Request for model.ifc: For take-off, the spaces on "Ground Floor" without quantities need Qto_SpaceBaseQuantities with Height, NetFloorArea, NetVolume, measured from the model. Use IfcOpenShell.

First a look at what the model holds.

```python
import ifcopenshell
import ifcopenshell.util.element
import ifcopenshell.util.unit

model = ifcopenshell.open("model.ifc")
print(model.schema)
for unit_type in ("LENGTHUNIT", "AREAUNIT", "VOLUMEUNIT"):
    print(unit_type, ifcopenshell.util.unit.calculate_unit_scale(model, unit_type))
storey = next(s for s in model.by_type("IfcBuildingStorey") if s.Name == "Ground Floor")
spaces = [e for e in ifcopenshell.util.element.get_decomposition(storey) if e.is_a("IfcSpace")]
for e in sorted(spaces, key=lambda e: e.id()):
    print(e.id(), e.is_a(), e.Name, list(ifcopenshell.util.element.get_psets(e, qtos_only=True)), sep=" | ")
```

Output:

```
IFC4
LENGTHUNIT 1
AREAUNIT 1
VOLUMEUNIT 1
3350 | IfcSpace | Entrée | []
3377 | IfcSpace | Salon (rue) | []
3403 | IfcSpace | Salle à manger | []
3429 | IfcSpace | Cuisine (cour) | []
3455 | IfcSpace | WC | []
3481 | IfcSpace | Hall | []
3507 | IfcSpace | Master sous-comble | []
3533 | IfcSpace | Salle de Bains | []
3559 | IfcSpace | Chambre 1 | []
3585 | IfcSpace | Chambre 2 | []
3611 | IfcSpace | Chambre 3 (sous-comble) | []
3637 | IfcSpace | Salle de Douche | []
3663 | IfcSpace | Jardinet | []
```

```python
import ifcopenshell
import ifcopenshell.api.pset
import ifcopenshell.geom
import ifcopenshell.util.element
import ifcopenshell.util.shape
import ifcopenshell.util.unit

model = ifcopenshell.open("model.ifc")
unit_scale = ifcopenshell.util.unit.calculate_unit_scale(model)
area_scale = ifcopenshell.util.unit.calculate_unit_scale(model, "AREAUNIT")
volume_scale = ifcopenshell.util.unit.calculate_unit_scale(model, "VOLUMEUNIT")
settings = ifcopenshell.geom.settings()

storey = next(s for s in model.by_type("IfcBuildingStorey") if s.Name == "Ground Floor")
spaces = [e for e in ifcopenshell.util.element.get_decomposition(storey) if e.is_a("IfcSpace")]

for e in sorted(spaces, key=lambda e: e.id()):
    if ifcopenshell.util.element.get_psets(e, qtos_only=True, should_inherit=False):
        continue
    # Geometry comes back in metres, in the element's own axes.
    shape = ifcopenshell.geom.create_shape(settings, e)
    values = {
        "Height": ifcopenshell.util.shape.get_z(shape.geometry) / unit_scale,
        "NetFloorArea": ifcopenshell.util.shape.get_footprint_area(shape.geometry) / area_scale,
        "NetVolume": ifcopenshell.util.shape.get_volume(shape.geometry) / volume_scale,
    }
    qto = ifcopenshell.api.pset.add_qto(model, product=e, name="Qto_SpaceBaseQuantities")
    ifcopenshell.api.pset.edit_qto(model, qto=qto, properties=values)
    print(e.id(), {k: round(v, 3) for k, v in values.items()})

model.write("model_updated.ifc")
```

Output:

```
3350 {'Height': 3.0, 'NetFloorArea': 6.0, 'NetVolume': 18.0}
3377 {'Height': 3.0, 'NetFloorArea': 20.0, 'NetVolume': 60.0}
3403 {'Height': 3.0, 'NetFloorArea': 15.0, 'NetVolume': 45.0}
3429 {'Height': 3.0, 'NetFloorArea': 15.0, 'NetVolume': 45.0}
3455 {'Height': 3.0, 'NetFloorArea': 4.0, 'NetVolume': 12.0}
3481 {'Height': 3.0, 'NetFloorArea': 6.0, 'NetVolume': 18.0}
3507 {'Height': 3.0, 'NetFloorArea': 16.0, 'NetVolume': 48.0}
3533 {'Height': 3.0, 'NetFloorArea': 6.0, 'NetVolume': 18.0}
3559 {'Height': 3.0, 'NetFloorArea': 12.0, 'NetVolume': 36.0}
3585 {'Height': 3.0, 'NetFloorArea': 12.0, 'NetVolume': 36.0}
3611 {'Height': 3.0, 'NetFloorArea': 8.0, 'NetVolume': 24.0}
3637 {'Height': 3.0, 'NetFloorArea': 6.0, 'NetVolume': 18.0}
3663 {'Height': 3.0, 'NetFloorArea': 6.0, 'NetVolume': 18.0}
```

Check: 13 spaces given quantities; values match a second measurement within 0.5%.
